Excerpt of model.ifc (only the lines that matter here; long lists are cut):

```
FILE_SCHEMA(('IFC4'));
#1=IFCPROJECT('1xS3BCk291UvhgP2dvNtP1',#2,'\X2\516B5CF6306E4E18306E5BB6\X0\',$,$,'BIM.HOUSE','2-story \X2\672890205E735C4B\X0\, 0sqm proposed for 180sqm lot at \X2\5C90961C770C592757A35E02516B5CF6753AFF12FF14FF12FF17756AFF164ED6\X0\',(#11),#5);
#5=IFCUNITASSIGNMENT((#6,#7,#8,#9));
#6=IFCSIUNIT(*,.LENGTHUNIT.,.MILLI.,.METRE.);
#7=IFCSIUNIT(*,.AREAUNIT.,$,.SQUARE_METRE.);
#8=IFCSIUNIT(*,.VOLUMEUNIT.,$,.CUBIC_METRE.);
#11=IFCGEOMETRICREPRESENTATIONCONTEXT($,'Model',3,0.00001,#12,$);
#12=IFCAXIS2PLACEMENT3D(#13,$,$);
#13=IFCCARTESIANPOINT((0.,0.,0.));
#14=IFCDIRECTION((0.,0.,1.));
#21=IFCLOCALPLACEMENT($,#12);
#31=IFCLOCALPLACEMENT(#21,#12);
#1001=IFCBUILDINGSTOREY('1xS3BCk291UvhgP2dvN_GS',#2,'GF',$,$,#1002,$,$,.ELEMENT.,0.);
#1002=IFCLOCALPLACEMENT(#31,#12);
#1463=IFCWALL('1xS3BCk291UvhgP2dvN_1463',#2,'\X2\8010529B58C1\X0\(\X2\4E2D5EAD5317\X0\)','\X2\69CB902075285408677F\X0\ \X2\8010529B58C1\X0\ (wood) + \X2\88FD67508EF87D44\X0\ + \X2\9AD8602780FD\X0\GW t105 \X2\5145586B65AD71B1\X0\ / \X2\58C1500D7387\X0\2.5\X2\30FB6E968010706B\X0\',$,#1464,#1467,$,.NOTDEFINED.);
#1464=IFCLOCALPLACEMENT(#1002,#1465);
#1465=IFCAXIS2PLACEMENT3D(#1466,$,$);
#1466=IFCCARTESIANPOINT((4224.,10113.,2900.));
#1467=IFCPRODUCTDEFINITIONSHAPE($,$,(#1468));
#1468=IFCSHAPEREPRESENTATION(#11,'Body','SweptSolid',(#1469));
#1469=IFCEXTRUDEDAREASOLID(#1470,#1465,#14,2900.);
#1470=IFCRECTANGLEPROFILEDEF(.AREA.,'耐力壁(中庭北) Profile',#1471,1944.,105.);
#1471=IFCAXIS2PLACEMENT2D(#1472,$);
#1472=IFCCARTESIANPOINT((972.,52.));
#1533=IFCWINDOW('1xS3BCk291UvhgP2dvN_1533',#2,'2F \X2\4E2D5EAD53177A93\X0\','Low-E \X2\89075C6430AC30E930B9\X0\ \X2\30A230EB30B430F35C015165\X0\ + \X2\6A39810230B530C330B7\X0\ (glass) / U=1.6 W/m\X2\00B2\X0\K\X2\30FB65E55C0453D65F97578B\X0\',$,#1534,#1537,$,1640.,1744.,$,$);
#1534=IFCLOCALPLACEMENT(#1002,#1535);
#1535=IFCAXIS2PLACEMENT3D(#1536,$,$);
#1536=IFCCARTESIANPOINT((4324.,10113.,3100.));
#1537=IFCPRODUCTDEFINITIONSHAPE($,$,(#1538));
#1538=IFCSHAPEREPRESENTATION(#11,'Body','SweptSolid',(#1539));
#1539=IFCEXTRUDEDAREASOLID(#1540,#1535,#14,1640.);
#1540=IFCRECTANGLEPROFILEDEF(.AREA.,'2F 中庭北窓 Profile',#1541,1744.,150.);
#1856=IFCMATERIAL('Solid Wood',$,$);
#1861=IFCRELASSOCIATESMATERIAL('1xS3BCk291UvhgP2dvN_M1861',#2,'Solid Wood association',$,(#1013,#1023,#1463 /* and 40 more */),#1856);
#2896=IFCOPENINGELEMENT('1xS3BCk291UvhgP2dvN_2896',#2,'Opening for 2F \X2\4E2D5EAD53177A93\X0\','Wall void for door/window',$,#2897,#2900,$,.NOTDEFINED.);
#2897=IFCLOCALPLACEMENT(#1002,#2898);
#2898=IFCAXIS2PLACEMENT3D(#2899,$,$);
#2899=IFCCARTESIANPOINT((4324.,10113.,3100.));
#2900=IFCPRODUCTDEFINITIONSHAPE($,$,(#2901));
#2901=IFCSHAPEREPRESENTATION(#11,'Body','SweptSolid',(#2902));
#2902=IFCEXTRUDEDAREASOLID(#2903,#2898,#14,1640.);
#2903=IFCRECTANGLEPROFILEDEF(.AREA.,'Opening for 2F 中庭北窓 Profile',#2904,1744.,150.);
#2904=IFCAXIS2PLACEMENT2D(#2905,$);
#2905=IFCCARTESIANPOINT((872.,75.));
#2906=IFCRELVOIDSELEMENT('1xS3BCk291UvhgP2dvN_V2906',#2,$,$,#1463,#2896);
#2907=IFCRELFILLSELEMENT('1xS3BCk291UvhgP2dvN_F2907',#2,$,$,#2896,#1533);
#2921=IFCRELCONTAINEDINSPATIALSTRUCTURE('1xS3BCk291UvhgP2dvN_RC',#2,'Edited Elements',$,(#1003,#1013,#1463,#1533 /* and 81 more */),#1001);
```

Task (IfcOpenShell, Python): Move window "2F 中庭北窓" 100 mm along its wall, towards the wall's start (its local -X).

```python
import ifcopenshell
import ifcopenshell.api.geometry
import ifcopenshell.util.placement

model = ifcopenshell.open("model.ifc")

window = model.by_guid("1xS3BCk291UvhgP2dvN_1533")
opening = window.FillsVoids[0].RelatingOpeningElement
wall = opening.VoidsElements[0].RelatingBuildingElement

wall_matrix = ifcopenshell.util.placement.get_local_placement(wall.ObjectPlacement)
shift = wall_matrix[:3, 0] * -100.0
before = ifcopenshell.util.placement.get_local_placement(window.ObjectPlacement)[:3, 3].copy()

# The window is not placed relative to its opening, so move both.
for product in (opening, window):
    matrix = ifcopenshell.util.placement.get_local_placement(product.ObjectPlacement)
    matrix[:3, 3] += shift
    ifcopenshell.api.geometry.edit_object_placement(model, product=product, matrix=matrix, is_si=False)

after = ifcopenshell.util.placement.get_local_placement(window.ObjectPlacement)[:3, 3]
print("window moved by", (after - before).round(3) + 0.0)

model.write("model_edited.ifc")
```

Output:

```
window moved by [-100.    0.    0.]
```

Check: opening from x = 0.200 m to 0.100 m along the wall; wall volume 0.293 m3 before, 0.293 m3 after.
